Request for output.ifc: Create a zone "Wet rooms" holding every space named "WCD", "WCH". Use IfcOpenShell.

First a look at what the model holds.

```python
import ifcopenshell

model = ifcopenshell.open("output.ifc")
print(model.schema)
seen = {}
for space in model.by_type("IfcSpace"):
    seen[space.LongName] = seen.get(space.LongName, 0) + 1
for name, count in sorted(seen.items(), key=str):
    print(count, "x", name)
print("zones:", [z.Name for z in model.by_type("IfcZone")][:20])
```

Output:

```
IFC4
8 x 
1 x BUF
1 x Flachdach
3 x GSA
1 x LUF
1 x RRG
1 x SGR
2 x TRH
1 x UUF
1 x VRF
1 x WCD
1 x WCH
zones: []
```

```python
import ifcopenshell
import ifcopenshell.api.group
import ifcopenshell.api.root

model = ifcopenshell.open("output.ifc")

names = {"WCD", "WCH"}
spaces = [s for s in model.by_type("IfcSpace") if s.LongName in names]

zone = ifcopenshell.api.root.create_entity(model, ifc_class="IfcZone", name="Wet rooms")
ifcopenshell.api.group.assign_group(model, products=spaces, group=zone)
print(len(spaces), "spaces in", zone.Name)

model.write("output-out.ifc")
```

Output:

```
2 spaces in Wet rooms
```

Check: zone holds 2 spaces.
